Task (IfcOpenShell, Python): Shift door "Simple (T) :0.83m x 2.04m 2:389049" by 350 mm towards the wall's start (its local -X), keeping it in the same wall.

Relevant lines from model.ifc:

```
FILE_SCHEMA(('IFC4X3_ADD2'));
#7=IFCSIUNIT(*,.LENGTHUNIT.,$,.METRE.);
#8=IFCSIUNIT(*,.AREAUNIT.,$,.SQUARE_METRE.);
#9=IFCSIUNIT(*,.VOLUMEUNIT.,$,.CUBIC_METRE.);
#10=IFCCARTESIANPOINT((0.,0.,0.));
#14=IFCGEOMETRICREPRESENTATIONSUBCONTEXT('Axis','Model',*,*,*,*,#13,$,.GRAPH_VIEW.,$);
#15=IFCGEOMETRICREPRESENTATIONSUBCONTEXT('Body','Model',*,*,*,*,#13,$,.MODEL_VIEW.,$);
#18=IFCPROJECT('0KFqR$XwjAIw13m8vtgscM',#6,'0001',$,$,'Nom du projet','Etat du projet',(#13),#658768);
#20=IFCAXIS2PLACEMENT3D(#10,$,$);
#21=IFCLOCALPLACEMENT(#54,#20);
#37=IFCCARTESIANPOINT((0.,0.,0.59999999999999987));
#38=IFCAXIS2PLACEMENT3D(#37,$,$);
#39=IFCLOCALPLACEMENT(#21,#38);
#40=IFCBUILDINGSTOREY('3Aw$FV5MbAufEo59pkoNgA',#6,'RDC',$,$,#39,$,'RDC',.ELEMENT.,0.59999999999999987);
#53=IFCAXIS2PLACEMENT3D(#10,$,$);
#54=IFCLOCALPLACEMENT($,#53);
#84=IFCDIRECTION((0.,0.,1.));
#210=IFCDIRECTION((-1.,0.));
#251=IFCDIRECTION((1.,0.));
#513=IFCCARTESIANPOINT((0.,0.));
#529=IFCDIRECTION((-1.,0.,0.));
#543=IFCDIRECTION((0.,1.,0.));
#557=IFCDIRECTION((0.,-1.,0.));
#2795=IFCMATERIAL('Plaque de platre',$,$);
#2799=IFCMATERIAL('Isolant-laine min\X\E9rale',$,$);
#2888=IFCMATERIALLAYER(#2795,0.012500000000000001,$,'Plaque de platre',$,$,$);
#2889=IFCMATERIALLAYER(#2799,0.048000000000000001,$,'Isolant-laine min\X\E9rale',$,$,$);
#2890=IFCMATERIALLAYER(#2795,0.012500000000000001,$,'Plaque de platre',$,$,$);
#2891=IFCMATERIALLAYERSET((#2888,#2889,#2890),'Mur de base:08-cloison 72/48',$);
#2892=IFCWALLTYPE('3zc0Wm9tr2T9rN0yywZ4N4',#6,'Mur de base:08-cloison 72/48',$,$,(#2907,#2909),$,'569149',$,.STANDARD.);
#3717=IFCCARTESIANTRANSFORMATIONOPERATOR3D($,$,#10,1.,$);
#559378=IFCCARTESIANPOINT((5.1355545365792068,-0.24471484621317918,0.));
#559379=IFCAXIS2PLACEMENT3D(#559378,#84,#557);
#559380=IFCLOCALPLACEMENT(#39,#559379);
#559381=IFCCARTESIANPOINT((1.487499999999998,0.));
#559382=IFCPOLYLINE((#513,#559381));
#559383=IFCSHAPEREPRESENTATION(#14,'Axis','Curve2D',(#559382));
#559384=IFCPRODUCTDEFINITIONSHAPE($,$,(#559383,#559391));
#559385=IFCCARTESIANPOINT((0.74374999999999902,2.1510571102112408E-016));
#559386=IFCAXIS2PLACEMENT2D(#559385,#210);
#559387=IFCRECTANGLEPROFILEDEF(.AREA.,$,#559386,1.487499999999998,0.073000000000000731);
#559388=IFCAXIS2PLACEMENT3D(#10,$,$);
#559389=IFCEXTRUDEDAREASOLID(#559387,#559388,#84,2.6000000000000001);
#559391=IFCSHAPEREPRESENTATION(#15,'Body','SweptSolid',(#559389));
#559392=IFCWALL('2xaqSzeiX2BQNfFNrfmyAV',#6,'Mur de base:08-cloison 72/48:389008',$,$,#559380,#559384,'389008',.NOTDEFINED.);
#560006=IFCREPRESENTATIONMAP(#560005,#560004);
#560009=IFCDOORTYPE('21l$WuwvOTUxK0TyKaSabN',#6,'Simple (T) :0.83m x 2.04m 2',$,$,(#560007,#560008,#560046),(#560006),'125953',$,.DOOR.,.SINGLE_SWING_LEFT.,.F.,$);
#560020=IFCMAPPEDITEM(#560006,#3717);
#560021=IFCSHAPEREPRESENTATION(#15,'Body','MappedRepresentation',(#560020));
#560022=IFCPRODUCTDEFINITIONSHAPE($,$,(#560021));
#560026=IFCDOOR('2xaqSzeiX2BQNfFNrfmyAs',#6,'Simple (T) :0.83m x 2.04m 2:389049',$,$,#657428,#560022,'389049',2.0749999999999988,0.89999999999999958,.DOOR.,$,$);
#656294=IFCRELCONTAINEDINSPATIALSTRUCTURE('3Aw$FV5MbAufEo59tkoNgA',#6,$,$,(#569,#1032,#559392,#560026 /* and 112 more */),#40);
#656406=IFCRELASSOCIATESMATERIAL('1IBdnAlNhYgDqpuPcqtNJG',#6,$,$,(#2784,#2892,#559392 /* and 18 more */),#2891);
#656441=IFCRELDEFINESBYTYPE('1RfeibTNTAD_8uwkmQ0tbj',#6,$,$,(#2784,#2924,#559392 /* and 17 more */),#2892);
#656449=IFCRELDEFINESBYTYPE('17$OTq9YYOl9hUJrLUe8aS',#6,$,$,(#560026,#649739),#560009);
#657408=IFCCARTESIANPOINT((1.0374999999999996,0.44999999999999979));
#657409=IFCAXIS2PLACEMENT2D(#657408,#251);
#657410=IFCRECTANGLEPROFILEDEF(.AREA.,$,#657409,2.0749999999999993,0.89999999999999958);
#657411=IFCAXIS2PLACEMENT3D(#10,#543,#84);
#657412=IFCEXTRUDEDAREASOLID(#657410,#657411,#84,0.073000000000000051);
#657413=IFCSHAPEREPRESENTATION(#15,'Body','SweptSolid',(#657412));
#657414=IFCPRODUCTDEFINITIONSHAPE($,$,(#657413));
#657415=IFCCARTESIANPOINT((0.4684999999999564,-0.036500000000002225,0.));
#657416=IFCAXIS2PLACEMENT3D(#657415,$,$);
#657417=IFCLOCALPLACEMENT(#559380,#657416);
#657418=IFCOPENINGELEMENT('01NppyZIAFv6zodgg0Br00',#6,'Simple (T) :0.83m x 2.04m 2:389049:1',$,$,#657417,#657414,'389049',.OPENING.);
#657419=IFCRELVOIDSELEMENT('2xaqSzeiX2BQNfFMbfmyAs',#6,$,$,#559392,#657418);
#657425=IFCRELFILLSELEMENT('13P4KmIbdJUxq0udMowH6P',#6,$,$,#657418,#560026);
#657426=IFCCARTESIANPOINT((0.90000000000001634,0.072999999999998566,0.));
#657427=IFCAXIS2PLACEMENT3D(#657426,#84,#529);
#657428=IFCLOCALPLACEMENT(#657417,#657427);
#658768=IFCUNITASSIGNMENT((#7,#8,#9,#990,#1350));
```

```python
import ifcopenshell
import ifcopenshell.api.geometry
import ifcopenshell.util.placement

model = ifcopenshell.open("model.ifc")

door = model.by_guid("2xaqSzeiX2BQNfFNrfmyAs")
opening = door.FillsVoids[0].RelatingOpeningElement
wall = opening.VoidsElements[0].RelatingBuildingElement

wall_matrix = ifcopenshell.util.placement.get_local_placement(wall.ObjectPlacement)
shift = wall_matrix[:3, 0] * -0.35
before = ifcopenshell.util.placement.get_local_placement(door.ObjectPlacement)[:3, 3].copy()

# The door is placed relative to its opening, so it follows when the opening moves.
matrix = ifcopenshell.util.placement.get_local_placement(opening.ObjectPlacement)
matrix[:3, 3] += shift
ifcopenshell.api.geometry.edit_object_placement(
    model, product=opening, matrix=matrix, is_si=False, should_transform_children=True
)

after = ifcopenshell.util.placement.get_local_placement(door.ObjectPlacement)[:3, 3]
print("door moved by", (after - before).round(3) + 0.0)

model.write("model_v2.ifc")
```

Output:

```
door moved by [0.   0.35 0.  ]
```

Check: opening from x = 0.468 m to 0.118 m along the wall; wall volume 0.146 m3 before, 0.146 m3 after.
